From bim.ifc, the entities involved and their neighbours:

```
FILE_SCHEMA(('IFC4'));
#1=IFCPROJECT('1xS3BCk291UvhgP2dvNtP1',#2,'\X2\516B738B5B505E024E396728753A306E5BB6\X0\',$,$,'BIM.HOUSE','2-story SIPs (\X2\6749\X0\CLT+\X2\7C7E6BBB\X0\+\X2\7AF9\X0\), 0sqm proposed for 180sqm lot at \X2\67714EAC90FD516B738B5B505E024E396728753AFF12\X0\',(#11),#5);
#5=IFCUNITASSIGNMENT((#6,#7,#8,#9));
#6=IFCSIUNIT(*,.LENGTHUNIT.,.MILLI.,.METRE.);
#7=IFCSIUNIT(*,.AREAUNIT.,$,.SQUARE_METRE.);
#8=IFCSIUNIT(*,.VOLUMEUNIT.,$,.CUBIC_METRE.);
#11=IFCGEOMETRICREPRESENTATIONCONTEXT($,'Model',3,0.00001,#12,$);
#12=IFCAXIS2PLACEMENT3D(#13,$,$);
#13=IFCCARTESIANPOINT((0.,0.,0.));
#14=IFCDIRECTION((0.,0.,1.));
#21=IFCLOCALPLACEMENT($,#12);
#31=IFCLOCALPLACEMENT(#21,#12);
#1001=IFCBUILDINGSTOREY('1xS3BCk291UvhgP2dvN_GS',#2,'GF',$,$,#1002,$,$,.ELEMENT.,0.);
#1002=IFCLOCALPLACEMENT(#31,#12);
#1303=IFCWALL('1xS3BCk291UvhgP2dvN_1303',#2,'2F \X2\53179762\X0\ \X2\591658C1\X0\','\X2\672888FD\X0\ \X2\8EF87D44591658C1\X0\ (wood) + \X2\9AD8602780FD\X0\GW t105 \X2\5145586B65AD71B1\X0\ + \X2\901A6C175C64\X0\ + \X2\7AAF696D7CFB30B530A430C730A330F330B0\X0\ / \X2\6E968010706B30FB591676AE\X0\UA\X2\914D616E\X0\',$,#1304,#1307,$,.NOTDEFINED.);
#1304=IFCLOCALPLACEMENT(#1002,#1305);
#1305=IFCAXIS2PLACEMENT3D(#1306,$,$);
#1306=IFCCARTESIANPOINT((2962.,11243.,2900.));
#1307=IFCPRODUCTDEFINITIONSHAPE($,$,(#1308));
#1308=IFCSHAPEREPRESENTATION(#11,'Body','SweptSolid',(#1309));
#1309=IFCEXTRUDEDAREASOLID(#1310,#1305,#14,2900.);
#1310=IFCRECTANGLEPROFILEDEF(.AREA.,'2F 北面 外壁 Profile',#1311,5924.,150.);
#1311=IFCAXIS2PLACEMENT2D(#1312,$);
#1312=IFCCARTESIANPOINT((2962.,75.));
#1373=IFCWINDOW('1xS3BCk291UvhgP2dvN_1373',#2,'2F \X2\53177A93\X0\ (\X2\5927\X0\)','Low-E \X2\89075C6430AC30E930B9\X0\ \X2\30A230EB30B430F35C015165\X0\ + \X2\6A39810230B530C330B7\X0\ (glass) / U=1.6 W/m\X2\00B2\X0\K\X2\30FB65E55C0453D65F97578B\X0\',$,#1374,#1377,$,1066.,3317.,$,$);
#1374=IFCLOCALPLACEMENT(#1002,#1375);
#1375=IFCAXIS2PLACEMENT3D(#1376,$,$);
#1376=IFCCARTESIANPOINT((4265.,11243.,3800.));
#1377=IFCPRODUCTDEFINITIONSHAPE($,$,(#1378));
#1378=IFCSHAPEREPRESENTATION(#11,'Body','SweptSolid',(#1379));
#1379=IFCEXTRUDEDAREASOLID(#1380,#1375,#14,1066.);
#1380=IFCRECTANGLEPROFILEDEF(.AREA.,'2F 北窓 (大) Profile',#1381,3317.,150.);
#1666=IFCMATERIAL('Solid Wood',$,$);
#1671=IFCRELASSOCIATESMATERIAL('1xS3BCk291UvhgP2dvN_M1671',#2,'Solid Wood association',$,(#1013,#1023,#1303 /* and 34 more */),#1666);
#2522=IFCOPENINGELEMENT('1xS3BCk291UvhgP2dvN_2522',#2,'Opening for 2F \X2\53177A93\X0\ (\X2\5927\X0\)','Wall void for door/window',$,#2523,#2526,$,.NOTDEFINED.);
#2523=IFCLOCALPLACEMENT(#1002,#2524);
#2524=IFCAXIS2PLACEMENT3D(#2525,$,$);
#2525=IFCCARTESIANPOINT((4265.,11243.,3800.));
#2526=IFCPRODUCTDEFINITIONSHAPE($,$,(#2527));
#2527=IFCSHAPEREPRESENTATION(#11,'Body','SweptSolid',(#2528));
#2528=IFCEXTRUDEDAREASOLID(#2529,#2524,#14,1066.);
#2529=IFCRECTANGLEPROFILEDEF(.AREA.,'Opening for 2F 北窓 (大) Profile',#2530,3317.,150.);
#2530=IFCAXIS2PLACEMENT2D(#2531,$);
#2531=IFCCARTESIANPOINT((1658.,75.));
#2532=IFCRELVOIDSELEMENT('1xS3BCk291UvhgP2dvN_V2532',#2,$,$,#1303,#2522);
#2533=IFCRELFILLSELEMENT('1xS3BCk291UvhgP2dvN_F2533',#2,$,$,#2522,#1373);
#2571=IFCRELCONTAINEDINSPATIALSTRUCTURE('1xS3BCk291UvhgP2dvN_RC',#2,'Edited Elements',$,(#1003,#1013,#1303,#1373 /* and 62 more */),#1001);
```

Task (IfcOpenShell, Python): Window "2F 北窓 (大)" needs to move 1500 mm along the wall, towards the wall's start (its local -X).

```python
import ifcopenshell
import ifcopenshell.api.geometry
import ifcopenshell.util.placement
import ifcopenshell.util.unit

model = ifcopenshell.open("bim.ifc")
unit_scale = ifcopenshell.util.unit.calculate_unit_scale(model)

window = model.by_guid("1xS3BCk291UvhgP2dvN_1373")
opening = window.FillsVoids[0].RelatingOpeningElement
wall = opening.VoidsElements[0].RelatingBuildingElement

wall_matrix = ifcopenshell.util.placement.get_local_placement(wall.ObjectPlacement)
shift = wall_matrix[:3, 0] * -1.5 / unit_scale
before = ifcopenshell.util.placement.get_local_placement(window.ObjectPlacement)[:3, 3].copy()

# The window is not placed relative to its opening, so move both.
for product in (opening, window):
    matrix = ifcopenshell.util.placement.get_local_placement(product.ObjectPlacement)
    matrix[:3, 3] += shift
    ifcopenshell.api.geometry.edit_object_placement(model, product=product, matrix=matrix, is_si=False)

after = ifcopenshell.util.placement.get_local_placement(window.ObjectPlacement)[:3, 3]
print("window moved by", (after - before).round(3) + 0.0)

model.write("bim_updated.ifc")
```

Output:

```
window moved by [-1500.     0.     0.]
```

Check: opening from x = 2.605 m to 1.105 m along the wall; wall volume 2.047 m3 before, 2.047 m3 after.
